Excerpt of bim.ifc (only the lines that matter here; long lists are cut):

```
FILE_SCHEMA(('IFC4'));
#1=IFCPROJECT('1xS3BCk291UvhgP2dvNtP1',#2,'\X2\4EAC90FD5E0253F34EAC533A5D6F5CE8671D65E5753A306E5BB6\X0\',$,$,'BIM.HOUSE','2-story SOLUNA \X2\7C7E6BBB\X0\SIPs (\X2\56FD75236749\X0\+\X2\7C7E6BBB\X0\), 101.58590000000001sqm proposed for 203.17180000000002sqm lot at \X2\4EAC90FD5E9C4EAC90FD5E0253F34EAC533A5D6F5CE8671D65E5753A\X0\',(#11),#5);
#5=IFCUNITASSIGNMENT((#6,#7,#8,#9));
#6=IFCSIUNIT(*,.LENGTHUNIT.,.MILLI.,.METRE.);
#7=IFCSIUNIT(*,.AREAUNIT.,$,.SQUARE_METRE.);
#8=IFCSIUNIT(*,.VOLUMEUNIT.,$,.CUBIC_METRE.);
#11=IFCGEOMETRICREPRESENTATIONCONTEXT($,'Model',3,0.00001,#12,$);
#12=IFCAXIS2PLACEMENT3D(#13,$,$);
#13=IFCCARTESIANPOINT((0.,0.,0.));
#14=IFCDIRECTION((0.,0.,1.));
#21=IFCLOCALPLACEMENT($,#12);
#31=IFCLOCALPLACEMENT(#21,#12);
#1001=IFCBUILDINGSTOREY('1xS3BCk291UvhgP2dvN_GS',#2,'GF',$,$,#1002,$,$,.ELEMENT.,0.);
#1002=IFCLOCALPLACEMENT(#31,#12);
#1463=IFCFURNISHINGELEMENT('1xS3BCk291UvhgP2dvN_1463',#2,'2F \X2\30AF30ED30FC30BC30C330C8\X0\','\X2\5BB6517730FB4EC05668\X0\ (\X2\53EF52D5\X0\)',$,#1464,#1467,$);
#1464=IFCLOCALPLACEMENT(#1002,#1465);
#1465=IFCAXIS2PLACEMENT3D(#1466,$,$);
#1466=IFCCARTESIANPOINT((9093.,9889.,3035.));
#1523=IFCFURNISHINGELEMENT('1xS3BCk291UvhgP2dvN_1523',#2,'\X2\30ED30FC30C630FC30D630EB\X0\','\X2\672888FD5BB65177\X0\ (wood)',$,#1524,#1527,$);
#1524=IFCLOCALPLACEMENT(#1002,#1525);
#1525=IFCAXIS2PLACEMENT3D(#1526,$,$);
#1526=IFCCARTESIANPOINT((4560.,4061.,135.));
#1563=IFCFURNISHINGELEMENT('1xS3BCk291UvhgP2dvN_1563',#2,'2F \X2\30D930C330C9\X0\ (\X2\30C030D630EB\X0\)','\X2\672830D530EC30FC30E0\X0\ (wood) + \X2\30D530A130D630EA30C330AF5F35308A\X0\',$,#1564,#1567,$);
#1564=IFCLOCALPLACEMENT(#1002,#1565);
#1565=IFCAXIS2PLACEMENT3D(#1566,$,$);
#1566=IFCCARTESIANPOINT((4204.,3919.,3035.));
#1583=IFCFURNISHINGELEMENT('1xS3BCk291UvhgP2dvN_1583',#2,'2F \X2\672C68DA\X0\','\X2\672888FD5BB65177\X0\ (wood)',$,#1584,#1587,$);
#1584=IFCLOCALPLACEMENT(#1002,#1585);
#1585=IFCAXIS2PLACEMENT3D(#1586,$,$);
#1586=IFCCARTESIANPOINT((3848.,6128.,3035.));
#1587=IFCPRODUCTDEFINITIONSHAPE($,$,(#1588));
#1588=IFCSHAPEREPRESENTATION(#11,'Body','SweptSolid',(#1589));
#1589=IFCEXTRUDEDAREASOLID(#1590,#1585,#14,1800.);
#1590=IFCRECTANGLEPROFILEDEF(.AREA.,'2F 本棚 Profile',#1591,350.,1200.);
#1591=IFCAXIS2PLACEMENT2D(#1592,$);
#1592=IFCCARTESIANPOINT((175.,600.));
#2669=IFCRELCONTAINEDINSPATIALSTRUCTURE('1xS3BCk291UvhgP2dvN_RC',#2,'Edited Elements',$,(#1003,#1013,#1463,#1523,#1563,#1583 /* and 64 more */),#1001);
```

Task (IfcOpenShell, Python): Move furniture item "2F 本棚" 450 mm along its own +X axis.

```python
import ifcopenshell
import ifcopenshell.api.geometry
import ifcopenshell.util.placement

model = ifcopenshell.open("bim.ifc")

item = model.by_guid("1xS3BCk291UvhgP2dvN_1583")
matrix = ifcopenshell.util.placement.get_local_placement(item.ObjectPlacement)
matrix[:3, 3] += matrix[:3, 0] * 450.0
ifcopenshell.api.geometry.edit_object_placement(model, product=item, matrix=matrix, is_si=False)

print(ifcopenshell.util.placement.get_local_placement(item.ObjectPlacement).round(3) + 0.0)

model.write("bim_rev.ifc")
```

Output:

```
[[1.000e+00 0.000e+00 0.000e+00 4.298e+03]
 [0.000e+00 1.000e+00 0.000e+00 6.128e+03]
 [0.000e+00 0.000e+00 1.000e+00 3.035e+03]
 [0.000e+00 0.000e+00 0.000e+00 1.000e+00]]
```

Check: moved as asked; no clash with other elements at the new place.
